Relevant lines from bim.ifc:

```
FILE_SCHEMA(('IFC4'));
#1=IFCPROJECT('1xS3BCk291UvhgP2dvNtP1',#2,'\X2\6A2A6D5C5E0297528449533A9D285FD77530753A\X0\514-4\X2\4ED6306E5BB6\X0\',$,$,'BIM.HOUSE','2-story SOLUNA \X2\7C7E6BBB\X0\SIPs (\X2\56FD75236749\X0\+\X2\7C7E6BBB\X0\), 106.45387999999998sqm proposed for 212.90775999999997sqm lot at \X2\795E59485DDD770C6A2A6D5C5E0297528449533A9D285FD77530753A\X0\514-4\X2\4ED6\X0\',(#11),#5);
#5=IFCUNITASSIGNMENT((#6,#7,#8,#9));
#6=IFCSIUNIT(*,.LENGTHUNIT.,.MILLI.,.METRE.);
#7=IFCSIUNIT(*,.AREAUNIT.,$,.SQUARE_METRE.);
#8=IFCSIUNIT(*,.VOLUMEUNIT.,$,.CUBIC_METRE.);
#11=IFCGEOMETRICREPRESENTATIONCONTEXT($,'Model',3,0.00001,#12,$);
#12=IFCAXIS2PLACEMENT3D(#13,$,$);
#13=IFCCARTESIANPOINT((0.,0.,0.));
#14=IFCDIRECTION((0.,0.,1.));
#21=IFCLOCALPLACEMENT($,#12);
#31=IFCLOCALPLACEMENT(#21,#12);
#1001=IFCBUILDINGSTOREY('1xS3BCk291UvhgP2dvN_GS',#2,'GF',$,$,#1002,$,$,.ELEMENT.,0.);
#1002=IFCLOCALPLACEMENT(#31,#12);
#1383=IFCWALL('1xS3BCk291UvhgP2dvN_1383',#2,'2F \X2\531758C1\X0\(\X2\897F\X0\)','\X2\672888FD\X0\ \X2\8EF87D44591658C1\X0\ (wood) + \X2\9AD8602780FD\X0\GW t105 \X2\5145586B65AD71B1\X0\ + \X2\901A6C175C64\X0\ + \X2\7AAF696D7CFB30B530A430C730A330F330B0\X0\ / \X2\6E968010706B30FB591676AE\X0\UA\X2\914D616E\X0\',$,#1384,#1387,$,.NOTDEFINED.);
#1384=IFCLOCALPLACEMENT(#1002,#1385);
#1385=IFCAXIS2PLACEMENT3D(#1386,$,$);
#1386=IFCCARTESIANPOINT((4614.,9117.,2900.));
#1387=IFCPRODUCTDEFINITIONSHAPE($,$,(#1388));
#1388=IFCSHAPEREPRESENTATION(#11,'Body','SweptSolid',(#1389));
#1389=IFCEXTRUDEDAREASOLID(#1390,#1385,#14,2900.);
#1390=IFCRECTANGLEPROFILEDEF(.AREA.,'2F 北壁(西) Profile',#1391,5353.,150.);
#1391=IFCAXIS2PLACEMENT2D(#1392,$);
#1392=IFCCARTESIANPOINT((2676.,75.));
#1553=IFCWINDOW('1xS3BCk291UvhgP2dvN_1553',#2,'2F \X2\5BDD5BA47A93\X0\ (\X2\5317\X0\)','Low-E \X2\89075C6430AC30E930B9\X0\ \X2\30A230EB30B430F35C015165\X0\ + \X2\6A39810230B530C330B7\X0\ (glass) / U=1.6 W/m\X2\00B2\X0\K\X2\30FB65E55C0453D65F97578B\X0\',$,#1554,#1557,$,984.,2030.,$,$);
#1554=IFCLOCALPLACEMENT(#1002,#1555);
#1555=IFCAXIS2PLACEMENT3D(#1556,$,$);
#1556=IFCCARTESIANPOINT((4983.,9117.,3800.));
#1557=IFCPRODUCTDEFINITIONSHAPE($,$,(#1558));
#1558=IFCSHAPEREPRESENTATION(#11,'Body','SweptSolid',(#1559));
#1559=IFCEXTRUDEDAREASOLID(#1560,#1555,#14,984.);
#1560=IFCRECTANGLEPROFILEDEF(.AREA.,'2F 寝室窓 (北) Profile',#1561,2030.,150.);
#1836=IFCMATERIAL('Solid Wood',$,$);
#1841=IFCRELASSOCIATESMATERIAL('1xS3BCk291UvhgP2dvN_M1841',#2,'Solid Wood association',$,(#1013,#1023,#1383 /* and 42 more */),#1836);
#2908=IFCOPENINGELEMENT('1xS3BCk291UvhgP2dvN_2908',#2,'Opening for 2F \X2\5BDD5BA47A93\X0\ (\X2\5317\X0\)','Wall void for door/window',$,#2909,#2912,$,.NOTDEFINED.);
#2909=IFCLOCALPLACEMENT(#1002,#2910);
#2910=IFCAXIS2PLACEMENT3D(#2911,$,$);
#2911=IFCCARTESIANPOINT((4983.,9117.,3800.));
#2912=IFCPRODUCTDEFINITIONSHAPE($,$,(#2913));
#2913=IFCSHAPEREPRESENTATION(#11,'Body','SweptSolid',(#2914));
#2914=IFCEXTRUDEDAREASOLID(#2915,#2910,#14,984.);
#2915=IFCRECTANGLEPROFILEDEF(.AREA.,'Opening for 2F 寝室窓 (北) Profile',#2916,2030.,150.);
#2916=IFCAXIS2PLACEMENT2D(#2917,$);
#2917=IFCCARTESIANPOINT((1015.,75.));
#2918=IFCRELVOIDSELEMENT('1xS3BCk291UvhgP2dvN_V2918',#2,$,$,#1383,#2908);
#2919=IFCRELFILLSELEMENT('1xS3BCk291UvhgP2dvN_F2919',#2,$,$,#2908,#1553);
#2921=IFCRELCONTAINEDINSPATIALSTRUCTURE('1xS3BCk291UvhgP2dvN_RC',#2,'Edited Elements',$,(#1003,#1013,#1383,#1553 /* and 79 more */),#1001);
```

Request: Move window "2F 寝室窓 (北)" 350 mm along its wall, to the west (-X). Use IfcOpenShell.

```python
import ifcopenshell
import ifcopenshell.api.geometry
import ifcopenshell.util.placement

model = ifcopenshell.open("bim.ifc")

window = model.by_guid("1xS3BCk291UvhgP2dvN_1553")
opening = window.FillsVoids[0].RelatingOpeningElement
wall = opening.VoidsElements[0].RelatingBuildingElement

wall_matrix = ifcopenshell.util.placement.get_local_placement(wall.ObjectPlacement)
shift = wall_matrix[:3, 0] * -350.0
before = ifcopenshell.util.placement.get_local_placement(window.ObjectPlacement)[:3, 3].copy()

# The window is not placed relative to its opening, so move both.
for product in (opening, window):
    matrix = ifcopenshell.util.placement.get_local_placement(product.ObjectPlacement)
    matrix[:3, 3] += shift
    ifcopenshell.api.geometry.edit_object_placement(model, product=product, matrix=matrix, is_si=False)

after = ifcopenshell.util.placement.get_local_placement(window.ObjectPlacement)[:3, 3]
print("window moved by", (after - before).round(3) + 0.0)

model.write("bim_rev.ifc")
```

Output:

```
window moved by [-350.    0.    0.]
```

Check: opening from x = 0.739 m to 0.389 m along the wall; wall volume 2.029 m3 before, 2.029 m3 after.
